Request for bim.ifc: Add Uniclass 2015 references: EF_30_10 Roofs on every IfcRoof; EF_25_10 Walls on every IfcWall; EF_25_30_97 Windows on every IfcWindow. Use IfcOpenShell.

First a look at what the model holds.

```python
import ifcopenshell

model = ifcopenshell.open("bim.ifc")
print(model.schema)
print("classifications:", [c.Name for c in model.by_type("IfcClassification")])
for ifc_class in ("IfcDoor", "IfcRoof", "IfcStair", "IfcWall", "IfcWindow"):
    print(ifc_class, len(model.by_type(ifc_class)))
```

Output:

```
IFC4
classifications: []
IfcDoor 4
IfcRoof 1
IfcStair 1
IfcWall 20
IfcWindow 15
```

```python
import ifcopenshell
import ifcopenshell.api.classification

model = ifcopenshell.open("bim.ifc")

system = ifcopenshell.api.classification.add_classification(model, classification="Uniclass 2015")

codes = {
    "IfcRoof": ("EF_30_10", "Roofs"),
    "IfcWall": ("EF_25_10", "Walls"),
    "IfcWindow": ("EF_25_30_97", "Windows"),
}
for ifc_class, (code, name) in codes.items():
    products = model.by_type(ifc_class)
    ifcopenshell.api.classification.add_reference(
        model, products=products, classification=system, identification=code, name=name
    )
    print(code, len(products))

model.write("bim_edited.ifc")
```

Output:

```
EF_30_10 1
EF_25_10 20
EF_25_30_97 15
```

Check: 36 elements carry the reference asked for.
